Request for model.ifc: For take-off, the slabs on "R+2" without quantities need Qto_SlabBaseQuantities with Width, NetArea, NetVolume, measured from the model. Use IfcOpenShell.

First a look at what the model holds.

```python
import ifcopenshell
import ifcopenshell.util.element
import ifcopenshell.util.unit

model = ifcopenshell.open("model.ifc")
print(model.schema)
for unit_type in ("LENGTHUNIT", "AREAUNIT", "VOLUMEUNIT"):
    print(unit_type, ifcopenshell.util.unit.calculate_unit_scale(model, unit_type))
storey = next(s for s in model.by_type("IfcBuildingStorey") if s.Name == "R+2")
slabs = [e for e in ifcopenshell.util.element.get_decomposition(storey) if e.is_a("IfcSlab")]
for e in sorted(slabs, key=lambda e: e.id()):
    print(e.id(), e.is_a(), e.Name, list(ifcopenshell.util.element.get_psets(e, qtos_only=True)), sep=" | ")
```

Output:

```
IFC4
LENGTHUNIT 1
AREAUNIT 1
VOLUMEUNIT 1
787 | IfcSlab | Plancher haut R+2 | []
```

```python
import ifcopenshell
import ifcopenshell.api.pset
import ifcopenshell.geom
import ifcopenshell.util.element
import ifcopenshell.util.shape
import ifcopenshell.util.unit

model = ifcopenshell.open("model.ifc")
unit_scale = ifcopenshell.util.unit.calculate_unit_scale(model)
area_scale = ifcopenshell.util.unit.calculate_unit_scale(model, "AREAUNIT")
volume_scale = ifcopenshell.util.unit.calculate_unit_scale(model, "VOLUMEUNIT")
settings = ifcopenshell.geom.settings()

storey = next(s for s in model.by_type("IfcBuildingStorey") if s.Name == "R+2")
slabs = [e for e in ifcopenshell.util.element.get_decomposition(storey) if e.is_a("IfcSlab")]

for e in sorted(slabs, key=lambda e: e.id()):
    if ifcopenshell.util.element.get_psets(e, qtos_only=True, should_inherit=False):
        continue
    # Geometry comes back in metres, in the element's own axes.
    shape = ifcopenshell.geom.create_shape(settings, e)
    values = {
        "Width": ifcopenshell.util.shape.get_z(shape.geometry) / unit_scale,
        "NetArea": ifcopenshell.util.shape.get_footprint_area(shape.geometry) / area_scale,
        "NetVolume": ifcopenshell.util.shape.get_volume(shape.geometry) / volume_scale,
    }
    qto = ifcopenshell.api.pset.add_qto(model, product=e, name="Qto_SlabBaseQuantities")
    ifcopenshell.api.pset.edit_qto(model, qto=qto, properties=values)
    print(e.id(), {k: round(v, 3) for k, v in values.items()})

model.write("model_edited.ifc")
```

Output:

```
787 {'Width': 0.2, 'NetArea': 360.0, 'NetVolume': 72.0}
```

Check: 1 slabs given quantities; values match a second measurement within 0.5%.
